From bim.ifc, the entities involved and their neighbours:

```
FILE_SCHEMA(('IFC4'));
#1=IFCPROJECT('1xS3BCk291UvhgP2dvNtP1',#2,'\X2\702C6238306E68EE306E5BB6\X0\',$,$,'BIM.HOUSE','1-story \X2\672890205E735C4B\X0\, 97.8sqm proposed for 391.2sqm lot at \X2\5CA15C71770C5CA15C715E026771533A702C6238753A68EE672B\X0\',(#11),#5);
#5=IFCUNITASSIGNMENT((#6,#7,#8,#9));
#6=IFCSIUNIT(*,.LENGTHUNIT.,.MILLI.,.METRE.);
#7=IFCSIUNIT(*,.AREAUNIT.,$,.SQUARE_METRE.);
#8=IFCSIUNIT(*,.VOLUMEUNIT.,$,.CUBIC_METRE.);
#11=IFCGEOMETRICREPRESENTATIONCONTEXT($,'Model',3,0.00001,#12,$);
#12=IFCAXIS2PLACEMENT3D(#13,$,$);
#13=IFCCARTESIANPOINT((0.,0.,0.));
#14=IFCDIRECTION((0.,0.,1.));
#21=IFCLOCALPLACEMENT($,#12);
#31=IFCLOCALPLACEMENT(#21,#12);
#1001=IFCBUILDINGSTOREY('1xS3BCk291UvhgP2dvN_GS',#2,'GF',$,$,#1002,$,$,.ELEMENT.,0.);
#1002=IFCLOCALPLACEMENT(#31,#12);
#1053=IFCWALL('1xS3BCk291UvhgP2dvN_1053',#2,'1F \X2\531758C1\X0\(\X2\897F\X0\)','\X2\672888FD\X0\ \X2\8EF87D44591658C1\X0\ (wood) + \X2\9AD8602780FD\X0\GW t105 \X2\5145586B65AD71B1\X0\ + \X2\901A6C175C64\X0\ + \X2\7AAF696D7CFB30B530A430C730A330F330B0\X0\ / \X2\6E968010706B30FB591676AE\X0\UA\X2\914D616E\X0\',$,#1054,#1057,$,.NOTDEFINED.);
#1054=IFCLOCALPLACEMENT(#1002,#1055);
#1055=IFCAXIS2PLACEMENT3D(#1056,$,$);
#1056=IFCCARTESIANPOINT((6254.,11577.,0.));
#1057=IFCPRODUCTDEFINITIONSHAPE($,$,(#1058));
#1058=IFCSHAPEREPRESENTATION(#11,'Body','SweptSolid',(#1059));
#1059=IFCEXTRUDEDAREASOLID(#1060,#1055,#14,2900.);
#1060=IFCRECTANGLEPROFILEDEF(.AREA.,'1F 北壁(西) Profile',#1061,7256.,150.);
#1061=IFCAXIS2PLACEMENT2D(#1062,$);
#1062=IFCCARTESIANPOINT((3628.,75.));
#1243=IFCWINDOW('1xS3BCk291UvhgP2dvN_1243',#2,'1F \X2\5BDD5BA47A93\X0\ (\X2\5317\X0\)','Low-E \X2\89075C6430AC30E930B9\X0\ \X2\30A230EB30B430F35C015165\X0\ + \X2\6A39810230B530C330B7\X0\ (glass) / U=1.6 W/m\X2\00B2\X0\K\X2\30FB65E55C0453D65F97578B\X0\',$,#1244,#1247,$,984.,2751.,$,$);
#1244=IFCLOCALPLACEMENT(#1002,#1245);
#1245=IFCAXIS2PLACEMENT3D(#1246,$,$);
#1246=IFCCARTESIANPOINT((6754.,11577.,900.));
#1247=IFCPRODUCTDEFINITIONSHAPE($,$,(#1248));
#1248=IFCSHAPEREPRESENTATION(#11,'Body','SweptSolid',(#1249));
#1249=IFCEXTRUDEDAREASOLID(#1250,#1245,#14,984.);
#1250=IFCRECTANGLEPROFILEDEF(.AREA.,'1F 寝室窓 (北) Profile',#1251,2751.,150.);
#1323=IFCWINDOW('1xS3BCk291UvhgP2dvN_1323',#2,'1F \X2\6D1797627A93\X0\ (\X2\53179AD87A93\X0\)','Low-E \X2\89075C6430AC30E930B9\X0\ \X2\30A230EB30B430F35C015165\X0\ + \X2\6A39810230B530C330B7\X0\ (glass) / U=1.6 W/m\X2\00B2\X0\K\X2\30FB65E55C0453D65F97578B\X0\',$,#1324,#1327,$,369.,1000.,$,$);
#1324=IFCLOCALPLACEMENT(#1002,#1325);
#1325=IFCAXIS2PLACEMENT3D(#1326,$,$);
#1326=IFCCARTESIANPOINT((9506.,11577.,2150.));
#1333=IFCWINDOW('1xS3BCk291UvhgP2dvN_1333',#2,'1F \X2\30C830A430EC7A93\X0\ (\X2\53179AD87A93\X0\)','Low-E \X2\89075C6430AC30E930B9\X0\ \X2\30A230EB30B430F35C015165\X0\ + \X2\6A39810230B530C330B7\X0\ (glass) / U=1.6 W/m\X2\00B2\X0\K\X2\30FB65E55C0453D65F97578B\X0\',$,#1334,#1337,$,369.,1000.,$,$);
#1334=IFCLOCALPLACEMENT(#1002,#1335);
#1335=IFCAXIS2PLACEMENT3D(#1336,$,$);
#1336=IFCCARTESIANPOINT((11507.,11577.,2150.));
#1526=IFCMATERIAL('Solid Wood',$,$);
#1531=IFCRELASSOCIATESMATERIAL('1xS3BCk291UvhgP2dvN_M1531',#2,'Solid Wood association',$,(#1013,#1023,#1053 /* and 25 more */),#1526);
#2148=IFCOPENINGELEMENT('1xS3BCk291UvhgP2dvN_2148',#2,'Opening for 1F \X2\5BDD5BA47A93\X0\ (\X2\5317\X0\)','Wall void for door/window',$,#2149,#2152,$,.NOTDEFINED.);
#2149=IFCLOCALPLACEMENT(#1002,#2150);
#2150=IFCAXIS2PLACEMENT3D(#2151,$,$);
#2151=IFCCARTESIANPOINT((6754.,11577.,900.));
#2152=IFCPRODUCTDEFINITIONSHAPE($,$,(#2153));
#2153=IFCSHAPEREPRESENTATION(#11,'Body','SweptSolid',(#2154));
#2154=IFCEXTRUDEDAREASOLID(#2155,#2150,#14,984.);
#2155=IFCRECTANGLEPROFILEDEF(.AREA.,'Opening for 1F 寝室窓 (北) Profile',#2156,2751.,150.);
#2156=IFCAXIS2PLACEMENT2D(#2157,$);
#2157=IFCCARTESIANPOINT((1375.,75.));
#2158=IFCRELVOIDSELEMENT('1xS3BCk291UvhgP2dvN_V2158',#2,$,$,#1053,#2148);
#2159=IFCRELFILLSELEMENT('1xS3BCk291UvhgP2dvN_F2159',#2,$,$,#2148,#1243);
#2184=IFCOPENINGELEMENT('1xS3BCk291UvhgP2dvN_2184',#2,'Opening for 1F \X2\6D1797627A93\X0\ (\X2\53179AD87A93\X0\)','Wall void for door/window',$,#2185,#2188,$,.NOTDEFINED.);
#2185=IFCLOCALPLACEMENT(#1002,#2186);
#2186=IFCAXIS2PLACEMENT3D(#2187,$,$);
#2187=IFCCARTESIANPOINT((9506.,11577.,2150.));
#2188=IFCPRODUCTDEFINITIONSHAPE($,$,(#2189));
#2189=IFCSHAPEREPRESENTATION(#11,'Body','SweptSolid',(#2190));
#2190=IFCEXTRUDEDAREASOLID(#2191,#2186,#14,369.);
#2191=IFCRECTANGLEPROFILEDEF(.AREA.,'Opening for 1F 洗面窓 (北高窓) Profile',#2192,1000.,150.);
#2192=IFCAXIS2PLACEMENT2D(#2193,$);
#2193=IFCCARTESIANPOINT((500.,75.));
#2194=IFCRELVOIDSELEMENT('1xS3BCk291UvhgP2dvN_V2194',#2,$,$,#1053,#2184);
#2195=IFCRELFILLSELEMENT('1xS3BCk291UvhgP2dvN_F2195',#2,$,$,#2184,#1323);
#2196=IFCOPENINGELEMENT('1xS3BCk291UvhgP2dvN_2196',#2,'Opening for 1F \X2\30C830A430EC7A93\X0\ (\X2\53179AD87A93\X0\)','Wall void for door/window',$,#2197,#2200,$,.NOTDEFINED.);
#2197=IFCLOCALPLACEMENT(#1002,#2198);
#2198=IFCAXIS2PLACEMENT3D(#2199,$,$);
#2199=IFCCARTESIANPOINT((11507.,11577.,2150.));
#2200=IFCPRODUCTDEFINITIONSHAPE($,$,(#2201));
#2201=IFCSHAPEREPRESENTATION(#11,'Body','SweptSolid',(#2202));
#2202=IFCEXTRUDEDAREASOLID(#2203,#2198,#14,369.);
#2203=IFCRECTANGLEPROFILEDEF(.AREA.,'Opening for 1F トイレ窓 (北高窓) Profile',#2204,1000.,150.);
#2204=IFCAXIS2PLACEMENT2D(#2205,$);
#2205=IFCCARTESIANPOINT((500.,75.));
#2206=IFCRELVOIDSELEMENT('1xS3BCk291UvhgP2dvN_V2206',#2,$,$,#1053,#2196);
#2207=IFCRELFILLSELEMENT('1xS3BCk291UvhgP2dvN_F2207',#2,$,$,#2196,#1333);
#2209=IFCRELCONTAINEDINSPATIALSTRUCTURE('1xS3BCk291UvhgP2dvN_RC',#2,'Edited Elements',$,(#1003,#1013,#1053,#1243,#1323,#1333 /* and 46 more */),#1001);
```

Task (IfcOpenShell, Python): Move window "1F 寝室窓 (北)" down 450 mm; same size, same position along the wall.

```python
import numpy as np
import ifcopenshell
import ifcopenshell.api.geometry
import ifcopenshell.util.placement
import ifcopenshell.util.unit

model = ifcopenshell.open("bim.ifc")
unit_scale = ifcopenshell.util.unit.calculate_unit_scale(model)

window = model.by_guid("1xS3BCk291UvhgP2dvN_1243")
opening = window.FillsVoids[0].RelatingOpeningElement
dz = -0.45 / unit_scale

shift = np.array([0.0, 0.0, dz])
# The window is not placed relative to its opening, so move both.
for product in (opening, window):
    matrix = ifcopenshell.util.placement.get_local_placement(product.ObjectPlacement)
    matrix[:3, 3] += shift
    ifcopenshell.api.geometry.edit_object_placement(model, product=product, matrix=matrix, is_si=False)

print(f"moved by {dz * unit_scale:+.3f} m")

model.write("bim_v2.ifc")
```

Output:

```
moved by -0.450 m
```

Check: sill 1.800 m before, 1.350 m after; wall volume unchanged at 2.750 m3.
